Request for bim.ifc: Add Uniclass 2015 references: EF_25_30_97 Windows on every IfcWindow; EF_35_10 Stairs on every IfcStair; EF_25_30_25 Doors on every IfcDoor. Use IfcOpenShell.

First a look at what the model holds.

```python
import ifcopenshell

model = ifcopenshell.open("bim.ifc")
print(model.schema)
print("classifications:", [c.Name for c in model.by_type("IfcClassification")])
for ifc_class in ("IfcDoor", "IfcRoof", "IfcStair", "IfcWall", "IfcWindow"):
    print(ifc_class, len(model.by_type(ifc_class)))
```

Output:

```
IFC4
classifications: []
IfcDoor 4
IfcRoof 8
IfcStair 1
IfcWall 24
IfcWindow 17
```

```python
import ifcopenshell
import ifcopenshell.api.classification

model = ifcopenshell.open("bim.ifc")

system = ifcopenshell.api.classification.add_classification(model, classification="Uniclass 2015")

codes = {
    "IfcWindow": ("EF_25_30_97", "Windows"),
    "IfcStair": ("EF_35_10", "Stairs"),
    "IfcDoor": ("EF_25_30_25", "Doors"),
}
for ifc_class, (code, name) in codes.items():
    products = model.by_type(ifc_class)
    ifcopenshell.api.classification.add_reference(
        model, products=products, classification=system, identification=code, name=name
    )
    print(code, len(products))

model.write("bim_edited.ifc")
```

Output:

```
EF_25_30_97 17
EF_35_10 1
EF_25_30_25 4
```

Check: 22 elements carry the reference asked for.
